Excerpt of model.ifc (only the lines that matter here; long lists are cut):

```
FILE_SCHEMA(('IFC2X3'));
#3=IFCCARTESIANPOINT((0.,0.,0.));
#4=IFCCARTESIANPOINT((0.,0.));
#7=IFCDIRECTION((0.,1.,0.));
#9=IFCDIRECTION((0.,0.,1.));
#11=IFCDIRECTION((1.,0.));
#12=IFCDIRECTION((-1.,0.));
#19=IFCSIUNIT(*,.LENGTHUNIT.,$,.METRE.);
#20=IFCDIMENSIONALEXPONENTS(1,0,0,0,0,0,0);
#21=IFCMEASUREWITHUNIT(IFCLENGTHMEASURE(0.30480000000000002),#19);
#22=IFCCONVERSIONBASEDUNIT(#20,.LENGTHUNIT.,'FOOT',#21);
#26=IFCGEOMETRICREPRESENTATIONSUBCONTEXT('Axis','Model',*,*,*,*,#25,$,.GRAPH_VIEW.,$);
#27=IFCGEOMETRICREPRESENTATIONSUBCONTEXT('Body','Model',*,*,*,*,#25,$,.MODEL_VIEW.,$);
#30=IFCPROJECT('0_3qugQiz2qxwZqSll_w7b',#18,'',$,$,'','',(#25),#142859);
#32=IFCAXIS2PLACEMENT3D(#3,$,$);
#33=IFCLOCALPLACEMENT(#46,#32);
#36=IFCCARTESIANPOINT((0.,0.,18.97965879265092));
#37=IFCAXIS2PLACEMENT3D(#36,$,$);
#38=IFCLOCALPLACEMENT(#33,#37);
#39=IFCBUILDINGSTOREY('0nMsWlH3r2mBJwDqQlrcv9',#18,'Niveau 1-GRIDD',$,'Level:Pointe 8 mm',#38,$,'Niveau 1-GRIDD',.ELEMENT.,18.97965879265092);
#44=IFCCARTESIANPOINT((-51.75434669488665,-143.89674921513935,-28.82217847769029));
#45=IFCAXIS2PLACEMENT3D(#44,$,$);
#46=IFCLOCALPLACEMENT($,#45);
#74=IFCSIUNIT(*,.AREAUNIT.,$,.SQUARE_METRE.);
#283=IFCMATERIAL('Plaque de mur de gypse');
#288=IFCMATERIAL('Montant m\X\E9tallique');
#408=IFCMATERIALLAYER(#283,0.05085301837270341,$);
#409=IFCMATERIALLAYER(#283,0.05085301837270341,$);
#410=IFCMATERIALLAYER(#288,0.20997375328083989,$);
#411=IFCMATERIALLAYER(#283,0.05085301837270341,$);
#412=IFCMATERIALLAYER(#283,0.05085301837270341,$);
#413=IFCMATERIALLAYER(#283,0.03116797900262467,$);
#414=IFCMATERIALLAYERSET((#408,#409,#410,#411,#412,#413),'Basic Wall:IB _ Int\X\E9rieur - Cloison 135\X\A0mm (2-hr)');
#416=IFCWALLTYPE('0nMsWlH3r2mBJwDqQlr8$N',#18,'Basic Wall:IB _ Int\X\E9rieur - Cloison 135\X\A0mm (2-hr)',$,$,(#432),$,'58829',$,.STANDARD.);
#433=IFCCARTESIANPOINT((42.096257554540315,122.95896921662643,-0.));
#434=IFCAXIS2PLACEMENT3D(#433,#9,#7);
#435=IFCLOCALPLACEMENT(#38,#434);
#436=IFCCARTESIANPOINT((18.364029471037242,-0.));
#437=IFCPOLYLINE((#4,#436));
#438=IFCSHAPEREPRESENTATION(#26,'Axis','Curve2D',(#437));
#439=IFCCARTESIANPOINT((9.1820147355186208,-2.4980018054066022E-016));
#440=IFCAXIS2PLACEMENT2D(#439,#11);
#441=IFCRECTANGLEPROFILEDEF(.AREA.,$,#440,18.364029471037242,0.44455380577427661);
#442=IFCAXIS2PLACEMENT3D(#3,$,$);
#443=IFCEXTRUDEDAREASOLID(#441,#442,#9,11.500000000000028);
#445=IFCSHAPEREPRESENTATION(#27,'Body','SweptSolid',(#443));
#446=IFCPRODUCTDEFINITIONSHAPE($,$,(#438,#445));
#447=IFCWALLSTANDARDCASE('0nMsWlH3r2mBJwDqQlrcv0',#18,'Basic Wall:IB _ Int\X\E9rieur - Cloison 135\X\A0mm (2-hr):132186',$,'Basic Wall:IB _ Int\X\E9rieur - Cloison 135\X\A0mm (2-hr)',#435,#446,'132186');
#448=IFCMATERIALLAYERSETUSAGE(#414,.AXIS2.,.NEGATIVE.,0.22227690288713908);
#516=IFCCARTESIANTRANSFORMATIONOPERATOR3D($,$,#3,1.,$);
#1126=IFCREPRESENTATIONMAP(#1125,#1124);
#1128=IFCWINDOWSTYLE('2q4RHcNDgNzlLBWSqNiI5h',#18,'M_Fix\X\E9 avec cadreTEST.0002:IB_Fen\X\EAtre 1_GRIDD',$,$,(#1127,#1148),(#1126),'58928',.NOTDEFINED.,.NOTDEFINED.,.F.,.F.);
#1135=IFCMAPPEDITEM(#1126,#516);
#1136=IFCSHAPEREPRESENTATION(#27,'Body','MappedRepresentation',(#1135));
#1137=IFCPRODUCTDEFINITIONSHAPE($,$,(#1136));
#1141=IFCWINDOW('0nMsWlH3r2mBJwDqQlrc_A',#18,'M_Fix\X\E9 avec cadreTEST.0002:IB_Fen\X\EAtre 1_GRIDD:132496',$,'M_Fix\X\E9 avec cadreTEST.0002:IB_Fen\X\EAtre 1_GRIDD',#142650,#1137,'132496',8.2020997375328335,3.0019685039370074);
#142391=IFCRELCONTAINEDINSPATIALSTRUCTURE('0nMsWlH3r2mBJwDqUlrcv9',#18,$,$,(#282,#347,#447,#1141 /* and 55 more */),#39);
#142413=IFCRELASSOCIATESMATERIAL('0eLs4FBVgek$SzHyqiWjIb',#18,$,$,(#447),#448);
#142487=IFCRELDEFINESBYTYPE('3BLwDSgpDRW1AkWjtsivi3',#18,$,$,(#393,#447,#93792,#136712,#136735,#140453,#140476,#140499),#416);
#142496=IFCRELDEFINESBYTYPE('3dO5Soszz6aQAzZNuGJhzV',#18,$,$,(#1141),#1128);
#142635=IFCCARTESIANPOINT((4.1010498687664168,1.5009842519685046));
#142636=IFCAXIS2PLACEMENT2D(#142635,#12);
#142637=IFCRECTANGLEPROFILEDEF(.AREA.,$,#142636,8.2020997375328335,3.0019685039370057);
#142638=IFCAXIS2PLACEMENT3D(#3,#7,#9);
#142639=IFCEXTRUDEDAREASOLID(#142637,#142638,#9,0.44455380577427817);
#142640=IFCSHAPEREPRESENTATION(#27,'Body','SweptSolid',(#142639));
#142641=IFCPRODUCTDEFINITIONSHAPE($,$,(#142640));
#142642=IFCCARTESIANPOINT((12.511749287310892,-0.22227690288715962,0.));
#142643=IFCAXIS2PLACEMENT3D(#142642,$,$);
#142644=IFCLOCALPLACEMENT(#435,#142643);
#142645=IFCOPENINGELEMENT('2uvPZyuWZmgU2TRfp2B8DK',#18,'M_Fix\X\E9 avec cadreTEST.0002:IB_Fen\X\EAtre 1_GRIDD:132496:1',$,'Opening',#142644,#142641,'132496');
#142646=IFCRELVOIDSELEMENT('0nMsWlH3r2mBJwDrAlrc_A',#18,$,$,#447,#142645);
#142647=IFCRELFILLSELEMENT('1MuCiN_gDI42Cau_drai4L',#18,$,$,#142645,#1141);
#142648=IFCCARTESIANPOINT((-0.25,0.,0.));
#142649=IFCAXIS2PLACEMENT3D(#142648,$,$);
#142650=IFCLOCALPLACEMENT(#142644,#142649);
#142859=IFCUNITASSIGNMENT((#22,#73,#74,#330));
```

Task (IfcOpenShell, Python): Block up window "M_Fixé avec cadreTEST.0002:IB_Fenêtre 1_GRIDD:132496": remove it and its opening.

```python
import ifcopenshell
import ifcopenshell.api.feature
import ifcopenshell.api.root
import ifcopenshell.geom
import ifcopenshell.util.shape

model = ifcopenshell.open("model.ifc")
settings = ifcopenshell.geom.settings()


def volume(element):
    """Net volume in cubic metres, openings subtracted."""
    shape = ifcopenshell.geom.create_shape(settings, element)
    return ifcopenshell.util.shape.get_volume(shape.geometry)


window = model.by_guid("0nMsWlH3r2mBJwDqQlrc_A")
opening = window.FillsVoids[0].RelatingOpeningElement
wall = opening.VoidsElements[0].RelatingBuildingElement
before = volume(wall)

ifcopenshell.api.root.remove_product(model, product=window)
ifcopenshell.api.feature.remove_feature(model, feature=opening)

after = volume(wall)

print(f"wall volume {before:.3f} -> {after:.3f} m3")

model.write("model_edited.ifc")
```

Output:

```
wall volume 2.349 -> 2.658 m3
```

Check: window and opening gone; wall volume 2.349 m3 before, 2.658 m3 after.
